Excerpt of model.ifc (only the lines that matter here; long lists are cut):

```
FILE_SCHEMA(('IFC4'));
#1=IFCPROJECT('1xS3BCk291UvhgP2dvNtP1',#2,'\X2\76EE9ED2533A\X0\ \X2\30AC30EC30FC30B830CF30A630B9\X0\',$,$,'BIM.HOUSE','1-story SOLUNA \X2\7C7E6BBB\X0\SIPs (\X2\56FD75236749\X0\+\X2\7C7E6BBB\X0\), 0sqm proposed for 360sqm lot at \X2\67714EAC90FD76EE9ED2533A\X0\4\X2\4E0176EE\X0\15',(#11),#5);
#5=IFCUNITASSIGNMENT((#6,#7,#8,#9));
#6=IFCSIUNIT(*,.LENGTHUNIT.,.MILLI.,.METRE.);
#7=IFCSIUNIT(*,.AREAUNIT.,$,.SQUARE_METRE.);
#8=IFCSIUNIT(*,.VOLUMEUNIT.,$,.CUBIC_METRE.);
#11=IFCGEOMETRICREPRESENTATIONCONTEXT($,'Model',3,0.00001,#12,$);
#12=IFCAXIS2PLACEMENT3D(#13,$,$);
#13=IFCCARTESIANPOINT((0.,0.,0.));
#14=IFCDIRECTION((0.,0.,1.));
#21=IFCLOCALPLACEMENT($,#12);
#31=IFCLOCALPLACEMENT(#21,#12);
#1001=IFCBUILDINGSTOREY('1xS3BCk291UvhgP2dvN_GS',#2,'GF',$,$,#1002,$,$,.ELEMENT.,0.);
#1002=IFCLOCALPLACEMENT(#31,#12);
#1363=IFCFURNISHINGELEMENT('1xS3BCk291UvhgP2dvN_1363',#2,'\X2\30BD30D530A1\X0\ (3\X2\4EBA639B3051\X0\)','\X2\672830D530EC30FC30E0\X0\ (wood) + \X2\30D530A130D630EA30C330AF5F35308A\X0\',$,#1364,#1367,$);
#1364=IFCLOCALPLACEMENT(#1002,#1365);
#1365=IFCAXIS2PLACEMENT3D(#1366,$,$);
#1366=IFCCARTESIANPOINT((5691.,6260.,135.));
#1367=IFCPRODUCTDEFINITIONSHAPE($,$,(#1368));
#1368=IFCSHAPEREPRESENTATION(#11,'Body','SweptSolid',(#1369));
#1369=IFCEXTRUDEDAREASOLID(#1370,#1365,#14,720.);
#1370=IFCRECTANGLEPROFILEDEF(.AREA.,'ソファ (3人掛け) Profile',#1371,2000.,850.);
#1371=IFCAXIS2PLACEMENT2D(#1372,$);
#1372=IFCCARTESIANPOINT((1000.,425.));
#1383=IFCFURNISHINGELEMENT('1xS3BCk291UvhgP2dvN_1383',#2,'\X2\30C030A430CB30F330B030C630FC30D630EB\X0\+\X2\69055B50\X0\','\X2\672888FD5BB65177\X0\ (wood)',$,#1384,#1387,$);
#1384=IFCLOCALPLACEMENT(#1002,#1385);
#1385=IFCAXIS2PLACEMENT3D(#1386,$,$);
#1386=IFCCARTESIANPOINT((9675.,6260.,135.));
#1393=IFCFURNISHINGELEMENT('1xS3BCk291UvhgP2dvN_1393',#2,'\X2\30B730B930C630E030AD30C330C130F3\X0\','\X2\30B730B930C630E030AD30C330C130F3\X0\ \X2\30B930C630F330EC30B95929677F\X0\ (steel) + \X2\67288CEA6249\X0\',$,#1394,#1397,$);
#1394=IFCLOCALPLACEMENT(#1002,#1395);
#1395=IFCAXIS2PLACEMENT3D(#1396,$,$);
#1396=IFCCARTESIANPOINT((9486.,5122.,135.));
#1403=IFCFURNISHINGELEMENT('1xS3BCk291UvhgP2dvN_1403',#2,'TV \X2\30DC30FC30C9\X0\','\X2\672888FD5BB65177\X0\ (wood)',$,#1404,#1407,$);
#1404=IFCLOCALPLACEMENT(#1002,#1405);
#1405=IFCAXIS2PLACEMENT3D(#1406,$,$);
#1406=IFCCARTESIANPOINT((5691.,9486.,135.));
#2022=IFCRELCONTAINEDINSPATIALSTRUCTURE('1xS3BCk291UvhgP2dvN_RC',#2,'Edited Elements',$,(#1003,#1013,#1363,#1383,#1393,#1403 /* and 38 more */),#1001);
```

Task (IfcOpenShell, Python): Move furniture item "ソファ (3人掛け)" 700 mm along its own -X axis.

```python
import ifcopenshell
import ifcopenshell.api.geometry
import ifcopenshell.util.placement

model = ifcopenshell.open("model.ifc")

item = model.by_guid("1xS3BCk291UvhgP2dvN_1363")
matrix = ifcopenshell.util.placement.get_local_placement(item.ObjectPlacement)
matrix[:3, 3] -= matrix[:3, 0] * 700.0
ifcopenshell.api.geometry.edit_object_placement(model, product=item, matrix=matrix, is_si=False)

print(ifcopenshell.util.placement.get_local_placement(item.ObjectPlacement).round(3) + 0.0)

model.write("model-out.ifc")
```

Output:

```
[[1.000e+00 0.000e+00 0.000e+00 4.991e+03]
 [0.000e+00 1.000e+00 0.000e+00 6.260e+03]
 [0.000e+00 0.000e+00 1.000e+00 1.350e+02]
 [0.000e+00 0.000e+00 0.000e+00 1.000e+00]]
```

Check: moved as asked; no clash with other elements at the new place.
